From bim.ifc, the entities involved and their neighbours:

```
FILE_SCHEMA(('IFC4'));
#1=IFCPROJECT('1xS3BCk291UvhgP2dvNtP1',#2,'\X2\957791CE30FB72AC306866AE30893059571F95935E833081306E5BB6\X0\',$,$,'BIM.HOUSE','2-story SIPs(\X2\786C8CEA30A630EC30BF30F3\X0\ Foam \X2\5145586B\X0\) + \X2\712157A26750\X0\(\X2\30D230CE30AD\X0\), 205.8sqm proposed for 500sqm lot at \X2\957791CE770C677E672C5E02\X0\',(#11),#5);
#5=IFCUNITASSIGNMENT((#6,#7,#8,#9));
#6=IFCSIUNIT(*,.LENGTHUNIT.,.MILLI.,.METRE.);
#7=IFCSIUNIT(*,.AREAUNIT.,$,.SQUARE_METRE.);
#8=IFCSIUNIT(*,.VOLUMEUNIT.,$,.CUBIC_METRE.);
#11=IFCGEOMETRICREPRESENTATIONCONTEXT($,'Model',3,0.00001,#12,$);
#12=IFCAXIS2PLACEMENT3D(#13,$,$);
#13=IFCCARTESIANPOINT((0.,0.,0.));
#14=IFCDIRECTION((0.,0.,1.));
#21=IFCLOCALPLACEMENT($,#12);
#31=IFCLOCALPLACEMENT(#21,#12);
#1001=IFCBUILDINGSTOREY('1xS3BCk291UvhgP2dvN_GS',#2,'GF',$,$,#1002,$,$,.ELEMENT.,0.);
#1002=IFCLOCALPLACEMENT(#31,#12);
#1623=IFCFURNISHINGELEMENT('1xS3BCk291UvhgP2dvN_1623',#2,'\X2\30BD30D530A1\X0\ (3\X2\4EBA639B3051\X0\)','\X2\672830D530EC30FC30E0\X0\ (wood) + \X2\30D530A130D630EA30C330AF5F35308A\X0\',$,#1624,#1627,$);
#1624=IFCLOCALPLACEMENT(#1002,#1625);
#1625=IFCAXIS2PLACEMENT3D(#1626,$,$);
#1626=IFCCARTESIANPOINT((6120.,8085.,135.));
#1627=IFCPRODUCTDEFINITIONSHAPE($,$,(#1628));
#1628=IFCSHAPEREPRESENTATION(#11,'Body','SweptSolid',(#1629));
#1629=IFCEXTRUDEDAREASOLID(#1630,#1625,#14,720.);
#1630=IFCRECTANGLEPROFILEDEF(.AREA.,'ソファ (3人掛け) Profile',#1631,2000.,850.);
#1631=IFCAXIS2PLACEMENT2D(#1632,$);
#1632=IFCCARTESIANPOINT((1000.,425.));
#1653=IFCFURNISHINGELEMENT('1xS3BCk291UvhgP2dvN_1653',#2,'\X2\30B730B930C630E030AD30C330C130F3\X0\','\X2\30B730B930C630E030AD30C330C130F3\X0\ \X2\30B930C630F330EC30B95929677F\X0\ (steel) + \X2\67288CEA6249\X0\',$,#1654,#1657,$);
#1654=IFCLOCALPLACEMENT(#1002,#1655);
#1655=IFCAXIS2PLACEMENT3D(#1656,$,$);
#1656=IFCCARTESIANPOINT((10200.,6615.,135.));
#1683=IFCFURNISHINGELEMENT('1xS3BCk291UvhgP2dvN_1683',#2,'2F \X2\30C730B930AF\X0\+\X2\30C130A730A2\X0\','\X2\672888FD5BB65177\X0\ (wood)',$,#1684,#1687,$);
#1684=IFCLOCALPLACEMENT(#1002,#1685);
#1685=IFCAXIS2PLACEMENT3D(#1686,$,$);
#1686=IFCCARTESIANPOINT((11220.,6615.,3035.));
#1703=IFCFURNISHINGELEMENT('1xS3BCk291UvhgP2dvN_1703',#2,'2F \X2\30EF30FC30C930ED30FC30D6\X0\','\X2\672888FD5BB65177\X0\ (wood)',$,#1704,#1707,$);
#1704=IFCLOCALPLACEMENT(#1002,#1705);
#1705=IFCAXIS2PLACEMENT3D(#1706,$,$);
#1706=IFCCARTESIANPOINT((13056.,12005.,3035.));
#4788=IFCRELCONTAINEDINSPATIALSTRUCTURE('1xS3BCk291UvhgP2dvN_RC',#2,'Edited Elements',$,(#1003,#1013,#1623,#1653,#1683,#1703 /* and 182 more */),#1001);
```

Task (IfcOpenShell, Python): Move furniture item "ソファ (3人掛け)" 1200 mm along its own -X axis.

```python
import ifcopenshell
import ifcopenshell.api.geometry
import ifcopenshell.util.placement

model = ifcopenshell.open("bim.ifc")

item = model.by_guid("1xS3BCk291UvhgP2dvN_1623")
matrix = ifcopenshell.util.placement.get_local_placement(item.ObjectPlacement)
matrix[:3, 3] -= matrix[:3, 0] * 1200.0
ifcopenshell.api.geometry.edit_object_placement(model, product=item, matrix=matrix, is_si=False)

print(ifcopenshell.util.placement.get_local_placement(item.ObjectPlacement).round(3) + 0.0)

model.write("bim-out.ifc")
```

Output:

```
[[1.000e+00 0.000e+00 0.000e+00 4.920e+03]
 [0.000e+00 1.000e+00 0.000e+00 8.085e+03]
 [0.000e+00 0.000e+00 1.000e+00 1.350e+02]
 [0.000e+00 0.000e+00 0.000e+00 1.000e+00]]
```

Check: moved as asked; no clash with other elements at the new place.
